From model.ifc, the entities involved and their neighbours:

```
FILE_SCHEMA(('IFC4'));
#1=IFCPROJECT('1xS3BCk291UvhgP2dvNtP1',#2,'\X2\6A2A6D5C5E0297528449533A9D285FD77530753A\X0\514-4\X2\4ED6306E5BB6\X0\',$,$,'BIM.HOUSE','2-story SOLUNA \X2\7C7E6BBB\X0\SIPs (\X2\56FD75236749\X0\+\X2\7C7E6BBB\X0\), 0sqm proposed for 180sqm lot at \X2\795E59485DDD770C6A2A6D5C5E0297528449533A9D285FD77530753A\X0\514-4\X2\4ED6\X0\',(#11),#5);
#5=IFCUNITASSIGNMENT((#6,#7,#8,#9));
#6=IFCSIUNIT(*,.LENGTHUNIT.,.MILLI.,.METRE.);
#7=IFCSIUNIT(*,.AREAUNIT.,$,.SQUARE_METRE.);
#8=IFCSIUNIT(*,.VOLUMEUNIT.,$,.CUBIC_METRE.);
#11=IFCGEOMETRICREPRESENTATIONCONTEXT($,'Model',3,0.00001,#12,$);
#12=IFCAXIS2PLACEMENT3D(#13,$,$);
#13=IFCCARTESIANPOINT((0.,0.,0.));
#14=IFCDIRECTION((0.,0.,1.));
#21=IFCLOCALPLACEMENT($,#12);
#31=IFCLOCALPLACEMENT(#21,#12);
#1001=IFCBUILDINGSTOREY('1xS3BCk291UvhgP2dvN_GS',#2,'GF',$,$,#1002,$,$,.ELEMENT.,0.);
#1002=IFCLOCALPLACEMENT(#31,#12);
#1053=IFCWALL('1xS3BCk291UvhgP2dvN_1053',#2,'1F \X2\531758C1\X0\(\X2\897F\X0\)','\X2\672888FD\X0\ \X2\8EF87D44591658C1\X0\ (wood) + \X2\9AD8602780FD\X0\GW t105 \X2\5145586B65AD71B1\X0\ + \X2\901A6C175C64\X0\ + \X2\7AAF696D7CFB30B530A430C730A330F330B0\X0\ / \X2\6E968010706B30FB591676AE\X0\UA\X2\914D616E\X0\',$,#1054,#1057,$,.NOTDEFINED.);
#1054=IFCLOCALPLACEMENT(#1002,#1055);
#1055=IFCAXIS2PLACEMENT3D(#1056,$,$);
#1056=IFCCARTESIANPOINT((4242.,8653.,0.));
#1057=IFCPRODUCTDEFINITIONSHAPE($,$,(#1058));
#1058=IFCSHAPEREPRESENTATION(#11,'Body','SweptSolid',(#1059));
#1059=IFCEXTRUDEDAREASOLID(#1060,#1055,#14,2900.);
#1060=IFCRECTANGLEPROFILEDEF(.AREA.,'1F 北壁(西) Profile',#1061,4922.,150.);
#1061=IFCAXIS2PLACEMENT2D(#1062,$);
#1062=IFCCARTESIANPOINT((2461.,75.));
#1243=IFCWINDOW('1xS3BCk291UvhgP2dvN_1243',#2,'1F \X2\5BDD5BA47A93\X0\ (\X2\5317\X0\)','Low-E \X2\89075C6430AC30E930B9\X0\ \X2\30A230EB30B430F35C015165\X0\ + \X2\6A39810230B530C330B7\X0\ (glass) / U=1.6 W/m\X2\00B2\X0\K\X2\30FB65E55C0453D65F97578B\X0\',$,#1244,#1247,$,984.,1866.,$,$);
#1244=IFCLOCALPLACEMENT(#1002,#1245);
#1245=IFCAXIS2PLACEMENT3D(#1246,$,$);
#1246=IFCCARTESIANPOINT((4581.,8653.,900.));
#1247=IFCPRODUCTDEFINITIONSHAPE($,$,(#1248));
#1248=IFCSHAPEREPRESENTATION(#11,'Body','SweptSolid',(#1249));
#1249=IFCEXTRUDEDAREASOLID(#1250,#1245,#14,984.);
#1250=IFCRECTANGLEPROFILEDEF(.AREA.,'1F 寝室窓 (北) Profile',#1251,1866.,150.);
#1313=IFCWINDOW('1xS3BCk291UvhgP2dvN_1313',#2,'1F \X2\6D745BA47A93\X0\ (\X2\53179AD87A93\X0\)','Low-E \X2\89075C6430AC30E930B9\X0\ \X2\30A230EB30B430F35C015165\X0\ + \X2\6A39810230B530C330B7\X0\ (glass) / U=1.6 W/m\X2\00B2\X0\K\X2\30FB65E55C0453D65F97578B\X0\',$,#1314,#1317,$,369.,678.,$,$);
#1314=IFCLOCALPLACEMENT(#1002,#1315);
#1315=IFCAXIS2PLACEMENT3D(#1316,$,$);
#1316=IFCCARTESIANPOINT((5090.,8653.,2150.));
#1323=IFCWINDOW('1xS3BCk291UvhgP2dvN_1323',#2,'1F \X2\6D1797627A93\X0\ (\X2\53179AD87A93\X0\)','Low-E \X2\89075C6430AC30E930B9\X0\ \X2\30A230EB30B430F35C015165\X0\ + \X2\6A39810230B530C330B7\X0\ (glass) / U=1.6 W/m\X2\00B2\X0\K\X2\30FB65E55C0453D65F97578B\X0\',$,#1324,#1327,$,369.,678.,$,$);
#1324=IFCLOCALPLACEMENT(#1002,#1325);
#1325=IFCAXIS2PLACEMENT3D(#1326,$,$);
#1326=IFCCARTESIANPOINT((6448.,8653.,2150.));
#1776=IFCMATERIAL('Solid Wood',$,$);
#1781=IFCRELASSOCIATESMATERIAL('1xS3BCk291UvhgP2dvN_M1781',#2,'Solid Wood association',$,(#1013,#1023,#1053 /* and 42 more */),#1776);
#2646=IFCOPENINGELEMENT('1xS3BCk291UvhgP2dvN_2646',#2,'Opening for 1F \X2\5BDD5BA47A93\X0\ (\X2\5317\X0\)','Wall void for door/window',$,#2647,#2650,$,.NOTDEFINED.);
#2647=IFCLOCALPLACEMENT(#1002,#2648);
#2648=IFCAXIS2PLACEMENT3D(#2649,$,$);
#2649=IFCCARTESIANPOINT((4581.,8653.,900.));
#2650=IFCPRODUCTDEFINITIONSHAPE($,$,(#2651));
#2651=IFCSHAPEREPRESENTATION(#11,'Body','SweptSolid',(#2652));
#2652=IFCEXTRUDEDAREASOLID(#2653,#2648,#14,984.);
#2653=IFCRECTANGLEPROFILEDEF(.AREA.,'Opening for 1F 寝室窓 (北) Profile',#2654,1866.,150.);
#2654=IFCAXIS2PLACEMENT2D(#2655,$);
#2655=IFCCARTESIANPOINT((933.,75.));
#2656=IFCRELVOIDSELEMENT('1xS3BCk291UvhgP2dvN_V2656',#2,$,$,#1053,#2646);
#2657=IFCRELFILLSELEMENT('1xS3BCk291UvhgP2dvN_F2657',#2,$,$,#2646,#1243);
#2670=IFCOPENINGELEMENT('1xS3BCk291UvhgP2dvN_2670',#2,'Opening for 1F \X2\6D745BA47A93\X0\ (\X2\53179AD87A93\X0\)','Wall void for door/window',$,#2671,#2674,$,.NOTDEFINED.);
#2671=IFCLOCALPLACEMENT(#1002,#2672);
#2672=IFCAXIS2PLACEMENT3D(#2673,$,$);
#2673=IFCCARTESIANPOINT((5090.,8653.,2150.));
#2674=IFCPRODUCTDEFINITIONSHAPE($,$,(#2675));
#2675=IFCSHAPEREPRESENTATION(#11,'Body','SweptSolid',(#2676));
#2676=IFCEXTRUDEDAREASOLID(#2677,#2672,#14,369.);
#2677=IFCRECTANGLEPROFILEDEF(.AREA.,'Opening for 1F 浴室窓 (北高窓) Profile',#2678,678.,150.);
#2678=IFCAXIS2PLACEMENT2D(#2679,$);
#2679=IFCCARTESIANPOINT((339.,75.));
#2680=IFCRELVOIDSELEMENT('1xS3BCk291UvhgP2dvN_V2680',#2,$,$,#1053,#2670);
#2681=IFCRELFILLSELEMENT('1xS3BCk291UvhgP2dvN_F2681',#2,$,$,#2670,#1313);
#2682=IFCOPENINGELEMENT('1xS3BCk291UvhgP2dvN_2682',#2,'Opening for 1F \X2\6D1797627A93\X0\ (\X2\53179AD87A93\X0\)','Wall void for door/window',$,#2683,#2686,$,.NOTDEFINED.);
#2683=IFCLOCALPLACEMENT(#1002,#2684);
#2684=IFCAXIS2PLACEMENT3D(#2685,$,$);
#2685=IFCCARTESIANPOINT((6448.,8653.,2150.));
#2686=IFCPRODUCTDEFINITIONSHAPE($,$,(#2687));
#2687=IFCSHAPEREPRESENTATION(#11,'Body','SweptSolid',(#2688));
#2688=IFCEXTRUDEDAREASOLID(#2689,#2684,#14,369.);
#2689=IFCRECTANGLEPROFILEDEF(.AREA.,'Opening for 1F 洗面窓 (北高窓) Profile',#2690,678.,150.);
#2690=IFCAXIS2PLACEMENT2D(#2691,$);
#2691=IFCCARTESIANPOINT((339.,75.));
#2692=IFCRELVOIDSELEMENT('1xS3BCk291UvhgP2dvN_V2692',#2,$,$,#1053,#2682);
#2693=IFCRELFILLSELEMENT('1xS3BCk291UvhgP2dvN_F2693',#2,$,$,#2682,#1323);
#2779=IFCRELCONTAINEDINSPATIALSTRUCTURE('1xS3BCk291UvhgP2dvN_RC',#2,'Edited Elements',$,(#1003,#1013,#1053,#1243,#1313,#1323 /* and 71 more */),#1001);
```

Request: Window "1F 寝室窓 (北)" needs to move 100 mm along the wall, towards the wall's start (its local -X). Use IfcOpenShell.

```python
import ifcopenshell
import ifcopenshell.api.geometry
import ifcopenshell.util.placement

model = ifcopenshell.open("model.ifc")

window = model.by_guid("1xS3BCk291UvhgP2dvN_1243")
opening = window.FillsVoids[0].RelatingOpeningElement
wall = opening.VoidsElements[0].RelatingBuildingElement

wall_matrix = ifcopenshell.util.placement.get_local_placement(wall.ObjectPlacement)
shift = wall_matrix[:3, 0] * -100.0
before = ifcopenshell.util.placement.get_local_placement(window.ObjectPlacement)[:3, 3].copy()

# The window is not placed relative to its opening, so move both.
for product in (opening, window):
    matrix = ifcopenshell.util.placement.get_local_placement(product.ObjectPlacement)
    matrix[:3, 3] += shift
    ifcopenshell.api.geometry.edit_object_placement(model, product=product, matrix=matrix, is_si=False)

after = ifcopenshell.util.placement.get_local_placement(window.ObjectPlacement)[:3, 3]
print("window moved by", (after - before).round(3) + 0.0)

model.write("model-out.ifc")
```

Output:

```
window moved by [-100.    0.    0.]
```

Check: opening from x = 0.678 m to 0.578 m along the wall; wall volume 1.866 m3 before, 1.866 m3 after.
